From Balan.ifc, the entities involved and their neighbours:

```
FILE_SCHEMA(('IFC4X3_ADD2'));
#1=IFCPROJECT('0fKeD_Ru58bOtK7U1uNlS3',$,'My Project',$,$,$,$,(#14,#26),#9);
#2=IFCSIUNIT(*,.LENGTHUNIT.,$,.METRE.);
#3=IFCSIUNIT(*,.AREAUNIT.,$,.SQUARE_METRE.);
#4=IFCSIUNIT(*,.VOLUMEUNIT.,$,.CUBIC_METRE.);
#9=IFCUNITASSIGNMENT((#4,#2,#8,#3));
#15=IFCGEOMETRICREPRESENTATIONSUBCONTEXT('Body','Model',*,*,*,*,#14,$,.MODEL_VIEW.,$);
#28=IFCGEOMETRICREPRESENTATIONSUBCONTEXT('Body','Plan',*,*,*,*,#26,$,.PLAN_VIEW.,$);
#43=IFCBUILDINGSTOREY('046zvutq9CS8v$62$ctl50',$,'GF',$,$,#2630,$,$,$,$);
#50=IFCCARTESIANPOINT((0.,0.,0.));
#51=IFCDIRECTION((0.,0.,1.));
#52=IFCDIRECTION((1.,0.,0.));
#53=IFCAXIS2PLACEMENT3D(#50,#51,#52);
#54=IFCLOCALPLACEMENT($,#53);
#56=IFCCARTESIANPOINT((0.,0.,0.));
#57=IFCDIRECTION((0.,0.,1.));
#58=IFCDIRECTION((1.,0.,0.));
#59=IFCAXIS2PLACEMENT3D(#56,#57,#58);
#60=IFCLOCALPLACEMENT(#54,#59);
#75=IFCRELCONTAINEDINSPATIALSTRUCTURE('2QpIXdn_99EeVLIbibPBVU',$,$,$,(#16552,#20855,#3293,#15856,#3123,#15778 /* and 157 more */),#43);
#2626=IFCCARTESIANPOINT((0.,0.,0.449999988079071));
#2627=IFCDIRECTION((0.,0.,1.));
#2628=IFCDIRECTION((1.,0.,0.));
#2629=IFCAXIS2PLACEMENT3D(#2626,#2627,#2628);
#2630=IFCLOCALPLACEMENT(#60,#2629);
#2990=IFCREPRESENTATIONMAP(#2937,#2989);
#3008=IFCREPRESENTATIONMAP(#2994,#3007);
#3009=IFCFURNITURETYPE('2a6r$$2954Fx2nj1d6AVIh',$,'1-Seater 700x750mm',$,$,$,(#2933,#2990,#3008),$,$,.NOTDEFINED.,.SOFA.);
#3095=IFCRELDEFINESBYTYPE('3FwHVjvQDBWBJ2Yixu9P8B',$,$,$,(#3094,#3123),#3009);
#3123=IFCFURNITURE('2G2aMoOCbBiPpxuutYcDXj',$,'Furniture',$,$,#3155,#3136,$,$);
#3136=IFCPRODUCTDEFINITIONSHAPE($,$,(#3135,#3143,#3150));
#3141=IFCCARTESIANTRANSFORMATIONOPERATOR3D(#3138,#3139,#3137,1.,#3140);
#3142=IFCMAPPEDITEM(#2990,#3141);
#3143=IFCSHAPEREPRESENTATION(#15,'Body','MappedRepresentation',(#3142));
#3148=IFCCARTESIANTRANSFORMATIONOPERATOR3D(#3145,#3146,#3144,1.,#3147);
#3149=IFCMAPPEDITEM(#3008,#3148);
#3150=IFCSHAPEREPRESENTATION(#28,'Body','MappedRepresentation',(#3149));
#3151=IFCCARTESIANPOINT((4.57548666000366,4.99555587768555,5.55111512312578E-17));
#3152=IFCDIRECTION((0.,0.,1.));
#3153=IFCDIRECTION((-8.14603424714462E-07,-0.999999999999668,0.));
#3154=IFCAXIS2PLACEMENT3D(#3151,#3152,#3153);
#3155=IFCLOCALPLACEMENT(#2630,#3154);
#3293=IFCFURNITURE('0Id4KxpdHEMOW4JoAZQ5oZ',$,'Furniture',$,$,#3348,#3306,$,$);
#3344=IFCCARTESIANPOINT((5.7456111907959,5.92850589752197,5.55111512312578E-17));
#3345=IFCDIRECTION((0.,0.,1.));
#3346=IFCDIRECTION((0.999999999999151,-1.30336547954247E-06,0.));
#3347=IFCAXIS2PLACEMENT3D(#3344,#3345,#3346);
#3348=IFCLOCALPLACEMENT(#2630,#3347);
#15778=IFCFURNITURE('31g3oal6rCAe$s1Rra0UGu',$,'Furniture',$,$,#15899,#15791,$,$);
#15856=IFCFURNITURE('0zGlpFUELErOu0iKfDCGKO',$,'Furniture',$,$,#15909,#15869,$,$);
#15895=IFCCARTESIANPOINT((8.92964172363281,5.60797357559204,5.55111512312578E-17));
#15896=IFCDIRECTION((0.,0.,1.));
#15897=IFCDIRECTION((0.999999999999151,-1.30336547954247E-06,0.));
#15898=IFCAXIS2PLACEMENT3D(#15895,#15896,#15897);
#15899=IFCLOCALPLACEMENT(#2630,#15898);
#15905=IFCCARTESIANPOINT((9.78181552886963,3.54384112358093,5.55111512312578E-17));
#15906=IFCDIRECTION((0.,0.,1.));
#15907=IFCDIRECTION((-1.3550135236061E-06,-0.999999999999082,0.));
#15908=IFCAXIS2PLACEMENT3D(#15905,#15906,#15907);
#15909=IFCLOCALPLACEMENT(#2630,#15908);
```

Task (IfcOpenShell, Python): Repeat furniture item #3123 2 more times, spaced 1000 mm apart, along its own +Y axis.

```python
import ifcopenshell
import ifcopenshell.api.geometry
import ifcopenshell.api.root
import ifcopenshell.util.element
import ifcopenshell.util.placement

model = ifcopenshell.open("Balan.ifc")

source = model.by_guid("2G2aMoOCbBiPpxuutYcDXj")
base = ifcopenshell.util.placement.get_local_placement(source.ObjectPlacement)
step = base[:3, 1] * 1.0

for i in range(1, 3):
    copy = ifcopenshell.api.root.copy_class(model, product=source)
    copy.Representation = ifcopenshell.util.element.copy_deep(
        model, source.Representation, exclude=["IfcGeometricRepresentationContext", "IfcRepresentationMap"]
    )
    matrix = base.copy()
    matrix[:3, 3] += i * step
    print("added at", matrix[:3, 3].round(3) + 0.0)
    ifcopenshell.api.geometry.edit_object_placement(model, product=copy, matrix=matrix, is_si=False)

model.write("Balan_edited.ifc")
```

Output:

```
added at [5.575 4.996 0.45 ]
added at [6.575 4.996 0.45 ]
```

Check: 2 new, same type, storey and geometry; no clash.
